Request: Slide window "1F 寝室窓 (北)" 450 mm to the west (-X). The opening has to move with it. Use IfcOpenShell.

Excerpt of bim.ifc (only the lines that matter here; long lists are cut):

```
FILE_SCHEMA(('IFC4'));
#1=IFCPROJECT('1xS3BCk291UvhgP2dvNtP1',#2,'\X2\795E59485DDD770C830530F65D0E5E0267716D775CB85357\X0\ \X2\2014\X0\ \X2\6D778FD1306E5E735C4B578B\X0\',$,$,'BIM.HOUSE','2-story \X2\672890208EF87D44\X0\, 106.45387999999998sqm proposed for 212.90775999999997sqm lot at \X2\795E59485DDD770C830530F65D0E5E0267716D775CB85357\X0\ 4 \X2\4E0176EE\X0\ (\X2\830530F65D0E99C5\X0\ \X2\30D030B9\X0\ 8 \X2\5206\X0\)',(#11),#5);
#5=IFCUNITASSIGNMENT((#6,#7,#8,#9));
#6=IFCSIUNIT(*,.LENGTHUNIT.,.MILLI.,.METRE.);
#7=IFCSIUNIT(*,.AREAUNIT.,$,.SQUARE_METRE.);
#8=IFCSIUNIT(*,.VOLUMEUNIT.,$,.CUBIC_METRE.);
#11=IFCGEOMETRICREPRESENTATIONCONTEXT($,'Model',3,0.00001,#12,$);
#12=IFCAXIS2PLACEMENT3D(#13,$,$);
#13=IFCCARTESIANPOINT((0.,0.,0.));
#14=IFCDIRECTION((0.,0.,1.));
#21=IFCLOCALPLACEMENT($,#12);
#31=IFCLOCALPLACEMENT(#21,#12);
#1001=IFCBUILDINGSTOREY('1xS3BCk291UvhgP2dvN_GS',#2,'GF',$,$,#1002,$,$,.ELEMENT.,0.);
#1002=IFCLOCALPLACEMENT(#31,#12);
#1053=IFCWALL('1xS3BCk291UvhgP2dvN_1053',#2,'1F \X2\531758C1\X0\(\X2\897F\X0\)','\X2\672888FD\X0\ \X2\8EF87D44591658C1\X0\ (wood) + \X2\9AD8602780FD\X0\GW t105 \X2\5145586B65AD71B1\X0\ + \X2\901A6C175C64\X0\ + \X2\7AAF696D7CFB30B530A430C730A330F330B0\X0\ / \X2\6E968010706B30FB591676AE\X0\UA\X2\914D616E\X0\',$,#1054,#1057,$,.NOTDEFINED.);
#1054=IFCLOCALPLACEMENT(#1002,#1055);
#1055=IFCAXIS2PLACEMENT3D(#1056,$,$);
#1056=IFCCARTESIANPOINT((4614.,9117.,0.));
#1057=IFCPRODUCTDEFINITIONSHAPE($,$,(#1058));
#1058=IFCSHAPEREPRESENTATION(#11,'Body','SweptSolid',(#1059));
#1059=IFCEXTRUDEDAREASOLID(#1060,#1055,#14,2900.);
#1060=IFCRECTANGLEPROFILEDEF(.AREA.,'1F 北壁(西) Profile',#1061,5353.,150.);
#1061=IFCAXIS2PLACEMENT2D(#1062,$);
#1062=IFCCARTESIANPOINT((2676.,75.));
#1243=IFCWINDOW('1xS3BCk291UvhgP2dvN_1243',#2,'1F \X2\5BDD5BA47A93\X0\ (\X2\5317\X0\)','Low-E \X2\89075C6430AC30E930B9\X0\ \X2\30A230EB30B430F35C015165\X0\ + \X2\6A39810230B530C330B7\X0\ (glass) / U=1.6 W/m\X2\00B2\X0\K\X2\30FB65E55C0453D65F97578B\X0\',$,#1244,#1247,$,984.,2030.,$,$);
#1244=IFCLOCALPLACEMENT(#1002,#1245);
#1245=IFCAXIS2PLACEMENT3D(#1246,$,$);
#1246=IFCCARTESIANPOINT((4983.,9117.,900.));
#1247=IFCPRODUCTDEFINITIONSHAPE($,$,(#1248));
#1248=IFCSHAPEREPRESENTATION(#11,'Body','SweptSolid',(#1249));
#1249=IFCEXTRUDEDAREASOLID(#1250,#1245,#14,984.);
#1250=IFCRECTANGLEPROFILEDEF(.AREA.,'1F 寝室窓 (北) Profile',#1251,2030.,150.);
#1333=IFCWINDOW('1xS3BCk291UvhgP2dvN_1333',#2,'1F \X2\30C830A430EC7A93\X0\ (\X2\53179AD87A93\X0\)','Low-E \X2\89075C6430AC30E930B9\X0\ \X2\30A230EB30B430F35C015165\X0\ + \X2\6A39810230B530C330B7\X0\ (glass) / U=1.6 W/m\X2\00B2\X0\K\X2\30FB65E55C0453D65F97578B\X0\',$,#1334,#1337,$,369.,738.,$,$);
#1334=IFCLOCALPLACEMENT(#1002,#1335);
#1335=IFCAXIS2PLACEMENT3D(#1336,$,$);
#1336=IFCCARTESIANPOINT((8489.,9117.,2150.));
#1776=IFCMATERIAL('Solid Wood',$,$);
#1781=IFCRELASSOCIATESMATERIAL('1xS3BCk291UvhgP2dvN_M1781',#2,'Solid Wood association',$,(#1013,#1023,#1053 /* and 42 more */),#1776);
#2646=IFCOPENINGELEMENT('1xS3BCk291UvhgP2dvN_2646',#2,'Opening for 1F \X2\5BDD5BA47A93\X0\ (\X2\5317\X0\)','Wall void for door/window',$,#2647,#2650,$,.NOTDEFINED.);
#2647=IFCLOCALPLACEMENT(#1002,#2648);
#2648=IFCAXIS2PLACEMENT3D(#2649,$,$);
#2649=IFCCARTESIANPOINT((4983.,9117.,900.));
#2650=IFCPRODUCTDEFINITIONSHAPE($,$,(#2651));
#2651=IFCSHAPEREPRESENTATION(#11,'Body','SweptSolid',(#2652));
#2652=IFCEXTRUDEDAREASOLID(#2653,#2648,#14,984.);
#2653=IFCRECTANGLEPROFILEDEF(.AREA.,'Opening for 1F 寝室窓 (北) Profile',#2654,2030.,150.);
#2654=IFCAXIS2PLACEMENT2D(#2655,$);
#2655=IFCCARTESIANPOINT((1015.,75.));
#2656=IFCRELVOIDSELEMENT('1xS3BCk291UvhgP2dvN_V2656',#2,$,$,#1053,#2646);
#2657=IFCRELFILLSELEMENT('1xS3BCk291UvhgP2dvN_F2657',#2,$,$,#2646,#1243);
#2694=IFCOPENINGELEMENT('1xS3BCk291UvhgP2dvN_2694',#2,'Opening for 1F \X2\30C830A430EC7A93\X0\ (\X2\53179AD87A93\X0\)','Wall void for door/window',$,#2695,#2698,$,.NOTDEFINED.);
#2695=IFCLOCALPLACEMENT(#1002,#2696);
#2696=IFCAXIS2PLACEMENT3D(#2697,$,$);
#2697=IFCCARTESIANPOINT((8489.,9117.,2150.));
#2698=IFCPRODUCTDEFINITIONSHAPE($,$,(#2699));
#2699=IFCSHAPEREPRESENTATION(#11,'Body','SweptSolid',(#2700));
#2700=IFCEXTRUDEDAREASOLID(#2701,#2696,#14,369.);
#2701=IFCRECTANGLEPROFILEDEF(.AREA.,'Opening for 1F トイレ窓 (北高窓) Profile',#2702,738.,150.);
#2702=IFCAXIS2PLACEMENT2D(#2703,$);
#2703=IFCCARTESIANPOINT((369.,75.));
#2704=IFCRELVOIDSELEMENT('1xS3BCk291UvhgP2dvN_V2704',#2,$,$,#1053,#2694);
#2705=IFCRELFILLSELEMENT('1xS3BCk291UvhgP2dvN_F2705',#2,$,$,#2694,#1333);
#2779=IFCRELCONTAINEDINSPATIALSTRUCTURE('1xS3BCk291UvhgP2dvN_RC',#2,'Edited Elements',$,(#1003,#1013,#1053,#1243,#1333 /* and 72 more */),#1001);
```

```python
import ifcopenshell
import ifcopenshell.api.geometry
import ifcopenshell.util.placement
import ifcopenshell.util.unit

model = ifcopenshell.open("bim.ifc")
unit_scale = ifcopenshell.util.unit.calculate_unit_scale(model)

window = model.by_guid("1xS3BCk291UvhgP2dvN_1243")
opening = window.FillsVoids[0].RelatingOpeningElement
wall = opening.VoidsElements[0].RelatingBuildingElement

wall_matrix = ifcopenshell.util.placement.get_local_placement(wall.ObjectPlacement)
shift = wall_matrix[:3, 0] * -0.45 / unit_scale
before = ifcopenshell.util.placement.get_local_placement(window.ObjectPlacement)[:3, 3].copy()

# The window is not placed relative to its opening, so move both.
for product in (opening, window):
    matrix = ifcopenshell.util.placement.get_local_placement(product.ObjectPlacement)
    matrix[:3, 3] += shift
    ifcopenshell.api.geometry.edit_object_placement(model, product=product, matrix=matrix, is_si=False)

after = ifcopenshell.util.placement.get_local_placement(window.ObjectPlacement)[:3, 3]
print("window moved by", (after - before).round(3) + 0.0)

model.write("bim_rev.ifc")
```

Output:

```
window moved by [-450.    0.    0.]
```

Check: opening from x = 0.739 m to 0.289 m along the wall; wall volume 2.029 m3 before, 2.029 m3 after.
